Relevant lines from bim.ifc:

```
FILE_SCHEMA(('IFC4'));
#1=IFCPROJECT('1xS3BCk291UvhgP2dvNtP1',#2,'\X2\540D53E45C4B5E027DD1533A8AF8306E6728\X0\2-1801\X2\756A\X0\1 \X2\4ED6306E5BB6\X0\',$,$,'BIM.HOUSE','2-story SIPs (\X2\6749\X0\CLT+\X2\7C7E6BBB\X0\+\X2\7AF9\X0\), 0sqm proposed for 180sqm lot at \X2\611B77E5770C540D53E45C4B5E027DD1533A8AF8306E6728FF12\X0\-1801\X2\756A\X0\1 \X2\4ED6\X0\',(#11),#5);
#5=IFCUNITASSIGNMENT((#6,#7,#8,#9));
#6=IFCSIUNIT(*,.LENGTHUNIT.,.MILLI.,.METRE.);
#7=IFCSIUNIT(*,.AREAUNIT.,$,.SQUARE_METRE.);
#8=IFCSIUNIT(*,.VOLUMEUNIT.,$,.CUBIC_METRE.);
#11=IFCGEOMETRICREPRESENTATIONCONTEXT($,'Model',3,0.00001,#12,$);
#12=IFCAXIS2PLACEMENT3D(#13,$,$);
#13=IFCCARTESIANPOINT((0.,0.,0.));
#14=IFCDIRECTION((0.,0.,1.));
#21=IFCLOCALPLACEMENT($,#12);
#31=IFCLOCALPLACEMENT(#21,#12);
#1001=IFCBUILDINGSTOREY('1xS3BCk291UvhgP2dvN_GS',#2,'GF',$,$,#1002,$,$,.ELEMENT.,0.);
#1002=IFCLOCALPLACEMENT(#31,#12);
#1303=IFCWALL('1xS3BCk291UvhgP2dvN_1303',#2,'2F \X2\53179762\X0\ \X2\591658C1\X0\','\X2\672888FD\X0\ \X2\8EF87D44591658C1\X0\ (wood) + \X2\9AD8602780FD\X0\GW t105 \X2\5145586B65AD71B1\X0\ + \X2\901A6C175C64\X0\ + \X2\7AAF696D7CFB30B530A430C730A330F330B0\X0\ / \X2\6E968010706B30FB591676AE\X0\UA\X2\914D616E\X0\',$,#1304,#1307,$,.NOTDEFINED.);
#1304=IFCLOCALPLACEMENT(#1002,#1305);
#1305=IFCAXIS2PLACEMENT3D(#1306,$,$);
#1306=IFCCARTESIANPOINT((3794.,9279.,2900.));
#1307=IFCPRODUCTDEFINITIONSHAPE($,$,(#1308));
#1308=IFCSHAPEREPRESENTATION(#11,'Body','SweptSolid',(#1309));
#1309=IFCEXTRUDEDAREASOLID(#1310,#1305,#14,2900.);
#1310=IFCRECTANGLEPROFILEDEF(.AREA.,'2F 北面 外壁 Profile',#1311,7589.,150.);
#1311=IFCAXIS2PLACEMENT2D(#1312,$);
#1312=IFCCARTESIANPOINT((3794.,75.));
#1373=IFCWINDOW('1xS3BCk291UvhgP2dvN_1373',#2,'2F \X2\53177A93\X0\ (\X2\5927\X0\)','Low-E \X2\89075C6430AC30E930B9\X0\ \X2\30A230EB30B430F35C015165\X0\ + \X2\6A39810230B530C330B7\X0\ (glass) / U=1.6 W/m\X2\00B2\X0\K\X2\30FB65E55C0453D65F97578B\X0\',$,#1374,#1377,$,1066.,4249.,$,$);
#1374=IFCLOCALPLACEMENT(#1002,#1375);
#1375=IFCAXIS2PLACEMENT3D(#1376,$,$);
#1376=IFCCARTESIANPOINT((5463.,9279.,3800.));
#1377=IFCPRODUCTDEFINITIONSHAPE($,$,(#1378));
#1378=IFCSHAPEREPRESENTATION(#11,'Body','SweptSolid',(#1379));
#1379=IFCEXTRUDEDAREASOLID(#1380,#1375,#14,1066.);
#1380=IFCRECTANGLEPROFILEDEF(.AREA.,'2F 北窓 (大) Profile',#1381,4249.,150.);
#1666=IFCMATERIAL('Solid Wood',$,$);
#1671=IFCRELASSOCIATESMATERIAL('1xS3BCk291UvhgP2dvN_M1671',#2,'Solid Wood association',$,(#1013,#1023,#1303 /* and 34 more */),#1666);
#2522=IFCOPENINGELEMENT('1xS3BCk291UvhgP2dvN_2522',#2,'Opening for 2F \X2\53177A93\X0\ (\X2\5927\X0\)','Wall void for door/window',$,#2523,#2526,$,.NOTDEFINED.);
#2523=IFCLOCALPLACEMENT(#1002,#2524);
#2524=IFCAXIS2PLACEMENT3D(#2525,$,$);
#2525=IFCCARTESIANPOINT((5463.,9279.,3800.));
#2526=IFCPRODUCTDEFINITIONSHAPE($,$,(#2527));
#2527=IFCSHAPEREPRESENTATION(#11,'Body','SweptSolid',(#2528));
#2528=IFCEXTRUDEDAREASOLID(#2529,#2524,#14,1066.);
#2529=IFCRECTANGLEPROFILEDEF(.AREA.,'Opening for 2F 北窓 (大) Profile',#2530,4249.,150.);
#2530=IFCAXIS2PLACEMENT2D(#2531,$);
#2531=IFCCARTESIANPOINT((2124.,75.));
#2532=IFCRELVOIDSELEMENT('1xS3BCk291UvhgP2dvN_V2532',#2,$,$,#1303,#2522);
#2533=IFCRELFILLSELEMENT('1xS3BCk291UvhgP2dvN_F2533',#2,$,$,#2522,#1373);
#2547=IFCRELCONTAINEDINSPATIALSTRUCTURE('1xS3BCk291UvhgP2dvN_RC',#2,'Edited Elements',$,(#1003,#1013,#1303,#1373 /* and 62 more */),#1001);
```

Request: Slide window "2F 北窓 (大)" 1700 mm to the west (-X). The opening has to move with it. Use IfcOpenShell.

```python
import ifcopenshell
import ifcopenshell.api.geometry
import ifcopenshell.util.placement

model = ifcopenshell.open("bim.ifc")

window = model.by_id(1373)
opening = window.FillsVoids[0].RelatingOpeningElement
wall = opening.VoidsElements[0].RelatingBuildingElement

wall_matrix = ifcopenshell.util.placement.get_local_placement(wall.ObjectPlacement)
shift = wall_matrix[:3, 0] * -1700.0
before = ifcopenshell.util.placement.get_local_placement(window.ObjectPlacement)[:3, 3].copy()

# The window is not placed relative to its opening, so move both.
for product in (opening, window):
    matrix = ifcopenshell.util.placement.get_local_placement(product.ObjectPlacement)
    matrix[:3, 3] += shift
    ifcopenshell.api.geometry.edit_object_placement(model, product=product, matrix=matrix, is_si=False)

after = ifcopenshell.util.placement.get_local_placement(window.ObjectPlacement)[:3, 3]
print("window moved by", (after - before).round(3) + 0.0)

model.write("bim-out.ifc")
```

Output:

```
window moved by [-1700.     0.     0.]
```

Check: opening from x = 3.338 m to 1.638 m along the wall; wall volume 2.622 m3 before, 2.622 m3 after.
